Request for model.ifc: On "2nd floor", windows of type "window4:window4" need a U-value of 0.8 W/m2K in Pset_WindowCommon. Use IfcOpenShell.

First a look at what the model holds.

```python
import ifcopenshell
import ifcopenshell.util.element

model = ifcopenshell.open("model.ifc")
print(model.schema)
storey = next(s for s in model.by_type("IfcBuildingStorey") if s.Name == "2nd floor")
windows = [e for e in ifcopenshell.util.element.get_decomposition(storey) if e.is_a("IfcWindow")]
seen = {}
for e in windows:
    element_type = ifcopenshell.util.element.get_type(e)
    key = (element_type.Name if element_type != e and element_type else None, ifcopenshell.util.element.get_pset(e, "Pset_WindowCommon", "ThermalTransmittance"))
    seen[key] = seen.get(key, 0) + 1
for (name, value), count in sorted(seen.items(), key=str):
    print(count, "x", name, "|", value)
```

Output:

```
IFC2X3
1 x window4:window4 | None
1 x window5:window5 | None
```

```python
import ifcopenshell
import ifcopenshell.api.pset
import ifcopenshell.util.element

model = ifcopenshell.open("model.ifc")

storey = next(s for s in model.by_type("IfcBuildingStorey") if s.Name == "2nd floor")
windows = [e for e in ifcopenshell.util.element.get_decomposition(storey) if e.is_a("IfcWindow")]

count = 0
for e in windows:
    element_type = ifcopenshell.util.element.get_type(e)
    if element_type in (None, e) or element_type.Name != "window4:window4":
        continue
    # add_pset returns the element's existing set when there is one.
    pset = ifcopenshell.api.pset.add_pset(model, product=e, name="Pset_WindowCommon")
    ifcopenshell.api.pset.edit_pset(model, pset=pset, properties={"ThermalTransmittance": 0.8})
    count += 1

print(count, "windows updated")

model.write("model_rev.ifc")
```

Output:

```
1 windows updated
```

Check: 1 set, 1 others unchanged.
